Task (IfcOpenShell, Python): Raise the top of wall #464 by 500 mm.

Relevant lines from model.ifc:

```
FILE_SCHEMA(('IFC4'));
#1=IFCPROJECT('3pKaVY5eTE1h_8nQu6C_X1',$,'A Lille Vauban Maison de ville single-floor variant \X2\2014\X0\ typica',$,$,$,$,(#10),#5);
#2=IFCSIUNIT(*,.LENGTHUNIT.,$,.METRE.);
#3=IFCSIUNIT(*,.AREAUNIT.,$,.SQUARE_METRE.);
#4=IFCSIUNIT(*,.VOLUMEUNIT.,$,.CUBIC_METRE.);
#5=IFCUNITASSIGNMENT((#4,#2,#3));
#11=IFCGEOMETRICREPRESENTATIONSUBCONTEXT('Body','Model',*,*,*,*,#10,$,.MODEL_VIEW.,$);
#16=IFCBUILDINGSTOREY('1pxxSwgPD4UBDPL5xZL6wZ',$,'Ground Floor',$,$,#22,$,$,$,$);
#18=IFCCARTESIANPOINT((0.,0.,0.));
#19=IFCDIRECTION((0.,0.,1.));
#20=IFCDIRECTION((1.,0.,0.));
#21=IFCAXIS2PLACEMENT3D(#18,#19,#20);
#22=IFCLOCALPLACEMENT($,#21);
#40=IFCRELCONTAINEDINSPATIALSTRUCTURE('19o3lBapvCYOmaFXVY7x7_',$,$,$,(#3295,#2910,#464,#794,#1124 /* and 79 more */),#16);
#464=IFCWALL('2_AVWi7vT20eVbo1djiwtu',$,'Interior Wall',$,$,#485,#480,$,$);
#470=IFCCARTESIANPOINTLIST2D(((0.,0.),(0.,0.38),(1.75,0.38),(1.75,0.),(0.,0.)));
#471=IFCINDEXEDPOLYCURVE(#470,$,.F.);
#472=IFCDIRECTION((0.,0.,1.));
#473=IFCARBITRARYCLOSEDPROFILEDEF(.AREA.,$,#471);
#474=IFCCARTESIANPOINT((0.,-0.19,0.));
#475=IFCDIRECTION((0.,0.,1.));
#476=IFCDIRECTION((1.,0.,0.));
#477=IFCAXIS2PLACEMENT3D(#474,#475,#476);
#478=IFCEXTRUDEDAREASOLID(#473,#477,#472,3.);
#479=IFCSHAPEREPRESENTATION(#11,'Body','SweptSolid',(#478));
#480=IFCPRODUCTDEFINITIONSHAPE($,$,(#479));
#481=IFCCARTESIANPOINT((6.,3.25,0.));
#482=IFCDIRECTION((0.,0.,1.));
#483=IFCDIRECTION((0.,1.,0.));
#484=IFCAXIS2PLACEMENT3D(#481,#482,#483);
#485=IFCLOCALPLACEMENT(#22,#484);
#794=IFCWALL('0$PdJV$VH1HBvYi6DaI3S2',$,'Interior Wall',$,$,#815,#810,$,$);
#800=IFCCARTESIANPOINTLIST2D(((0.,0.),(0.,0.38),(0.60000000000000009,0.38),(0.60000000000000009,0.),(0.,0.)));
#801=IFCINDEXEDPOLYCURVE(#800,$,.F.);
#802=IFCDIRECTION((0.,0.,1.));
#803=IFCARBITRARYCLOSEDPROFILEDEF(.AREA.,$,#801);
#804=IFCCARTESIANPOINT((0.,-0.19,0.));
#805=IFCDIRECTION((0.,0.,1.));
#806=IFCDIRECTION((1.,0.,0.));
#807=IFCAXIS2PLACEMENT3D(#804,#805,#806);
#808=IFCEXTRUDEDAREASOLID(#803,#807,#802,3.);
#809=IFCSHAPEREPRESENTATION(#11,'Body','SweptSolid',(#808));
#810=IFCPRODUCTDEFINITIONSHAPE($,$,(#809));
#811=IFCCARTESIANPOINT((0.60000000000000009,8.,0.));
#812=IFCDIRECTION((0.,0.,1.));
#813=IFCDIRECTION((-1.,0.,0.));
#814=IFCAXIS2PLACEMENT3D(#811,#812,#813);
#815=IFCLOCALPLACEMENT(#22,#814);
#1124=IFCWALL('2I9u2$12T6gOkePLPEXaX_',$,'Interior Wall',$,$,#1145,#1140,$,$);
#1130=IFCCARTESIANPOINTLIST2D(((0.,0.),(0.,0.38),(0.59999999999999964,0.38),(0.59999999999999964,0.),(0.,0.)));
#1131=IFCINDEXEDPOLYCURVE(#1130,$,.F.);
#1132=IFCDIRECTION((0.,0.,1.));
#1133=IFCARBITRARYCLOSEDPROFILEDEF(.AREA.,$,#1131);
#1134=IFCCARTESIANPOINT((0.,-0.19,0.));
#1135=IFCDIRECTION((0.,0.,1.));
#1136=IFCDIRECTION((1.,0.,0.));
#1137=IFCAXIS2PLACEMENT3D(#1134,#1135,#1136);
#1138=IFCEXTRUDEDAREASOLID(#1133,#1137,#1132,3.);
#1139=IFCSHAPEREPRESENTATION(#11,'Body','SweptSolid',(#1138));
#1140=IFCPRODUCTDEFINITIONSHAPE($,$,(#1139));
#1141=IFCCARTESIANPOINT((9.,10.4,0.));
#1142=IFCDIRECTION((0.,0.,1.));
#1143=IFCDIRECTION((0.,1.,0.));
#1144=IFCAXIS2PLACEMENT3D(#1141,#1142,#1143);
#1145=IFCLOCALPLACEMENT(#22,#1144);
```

```python
import ifcopenshell
import ifcopenshell.geom
import ifcopenshell.util.representation
import ifcopenshell.util.shape

model = ifcopenshell.open("model.ifc")
settings = ifcopenshell.geom.settings()


def volume(element):
    """Net volume in cubic metres, openings subtracted."""
    shape = ifcopenshell.geom.create_shape(settings, element)
    return ifcopenshell.util.shape.get_volume(shape.geometry)


wall = model.by_guid("2_AVWi7vT20eVbo1djiwtu")
before = volume(wall)

body = ifcopenshell.util.representation.get_representation(wall, "Model", "Body")
solid = body.Items[0]
old_height = solid.Depth
solid.Depth += 0.5
after = volume(wall)

print(f"height {old_height:g} -> {solid.Depth:g}, volume {before:.3f} -> {after:.3f} m3")

model.write("model_rev.ifc")
```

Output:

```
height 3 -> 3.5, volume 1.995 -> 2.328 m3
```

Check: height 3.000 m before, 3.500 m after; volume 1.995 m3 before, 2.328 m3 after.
